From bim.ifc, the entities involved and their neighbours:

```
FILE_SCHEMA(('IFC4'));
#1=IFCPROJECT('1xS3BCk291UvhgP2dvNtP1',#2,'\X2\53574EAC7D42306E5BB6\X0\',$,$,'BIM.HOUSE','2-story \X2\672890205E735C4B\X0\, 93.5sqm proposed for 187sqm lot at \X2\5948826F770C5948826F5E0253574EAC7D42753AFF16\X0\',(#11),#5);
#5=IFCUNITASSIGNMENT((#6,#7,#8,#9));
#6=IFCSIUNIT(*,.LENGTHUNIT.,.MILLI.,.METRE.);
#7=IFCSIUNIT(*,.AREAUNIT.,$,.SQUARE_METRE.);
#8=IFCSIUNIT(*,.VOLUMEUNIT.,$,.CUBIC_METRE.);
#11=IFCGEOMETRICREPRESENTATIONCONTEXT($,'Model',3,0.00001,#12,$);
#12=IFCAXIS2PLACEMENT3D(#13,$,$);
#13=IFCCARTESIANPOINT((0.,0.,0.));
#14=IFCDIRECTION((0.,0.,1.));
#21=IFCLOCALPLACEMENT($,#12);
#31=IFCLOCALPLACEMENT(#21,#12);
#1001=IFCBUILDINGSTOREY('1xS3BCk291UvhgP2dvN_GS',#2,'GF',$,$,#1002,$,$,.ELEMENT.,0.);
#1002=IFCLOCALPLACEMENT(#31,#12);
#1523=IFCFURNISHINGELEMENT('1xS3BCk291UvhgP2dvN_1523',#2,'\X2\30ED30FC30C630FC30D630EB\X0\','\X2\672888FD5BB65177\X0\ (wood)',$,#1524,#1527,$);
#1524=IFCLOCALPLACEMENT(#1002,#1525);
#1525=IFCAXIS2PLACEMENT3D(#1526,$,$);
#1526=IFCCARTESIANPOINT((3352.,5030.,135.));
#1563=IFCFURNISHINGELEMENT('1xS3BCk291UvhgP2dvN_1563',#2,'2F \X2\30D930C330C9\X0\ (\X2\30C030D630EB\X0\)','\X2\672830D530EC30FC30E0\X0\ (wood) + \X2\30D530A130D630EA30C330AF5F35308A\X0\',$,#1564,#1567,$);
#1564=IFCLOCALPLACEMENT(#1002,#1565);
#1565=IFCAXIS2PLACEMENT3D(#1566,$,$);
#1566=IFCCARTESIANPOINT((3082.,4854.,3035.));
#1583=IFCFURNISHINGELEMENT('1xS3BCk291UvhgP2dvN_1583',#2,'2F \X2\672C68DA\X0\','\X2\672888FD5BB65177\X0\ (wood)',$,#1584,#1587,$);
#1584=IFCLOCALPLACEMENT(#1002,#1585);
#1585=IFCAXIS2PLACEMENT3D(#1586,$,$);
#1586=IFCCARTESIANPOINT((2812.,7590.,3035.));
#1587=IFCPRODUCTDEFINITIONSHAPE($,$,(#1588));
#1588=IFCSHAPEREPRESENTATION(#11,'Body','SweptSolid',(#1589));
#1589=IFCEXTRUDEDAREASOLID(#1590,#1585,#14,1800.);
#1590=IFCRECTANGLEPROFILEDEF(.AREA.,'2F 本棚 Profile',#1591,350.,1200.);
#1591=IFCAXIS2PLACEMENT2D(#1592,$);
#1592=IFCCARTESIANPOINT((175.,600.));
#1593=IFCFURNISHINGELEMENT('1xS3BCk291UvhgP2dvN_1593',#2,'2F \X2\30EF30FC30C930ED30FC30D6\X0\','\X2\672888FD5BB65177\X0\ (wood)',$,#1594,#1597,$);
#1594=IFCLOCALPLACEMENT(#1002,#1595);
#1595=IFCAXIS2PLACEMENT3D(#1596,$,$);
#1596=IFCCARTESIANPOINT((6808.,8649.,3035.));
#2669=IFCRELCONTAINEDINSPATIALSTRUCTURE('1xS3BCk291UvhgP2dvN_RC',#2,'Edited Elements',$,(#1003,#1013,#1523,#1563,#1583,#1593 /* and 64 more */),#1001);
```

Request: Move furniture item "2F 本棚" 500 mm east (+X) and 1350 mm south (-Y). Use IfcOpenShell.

```python
import ifcopenshell
import ifcopenshell.api.geometry
import ifcopenshell.util.placement

model = ifcopenshell.open("bim.ifc")

item = model.by_guid("1xS3BCk291UvhgP2dvN_1583")
matrix = ifcopenshell.util.placement.get_local_placement(item.ObjectPlacement)
matrix[0, 3] += 500.0
matrix[1, 3] -= 1350.0
ifcopenshell.api.geometry.edit_object_placement(model, product=item, matrix=matrix, is_si=False)

print(ifcopenshell.util.placement.get_local_placement(item.ObjectPlacement).round(3) + 0.0)

model.write("bim_updated.ifc")
```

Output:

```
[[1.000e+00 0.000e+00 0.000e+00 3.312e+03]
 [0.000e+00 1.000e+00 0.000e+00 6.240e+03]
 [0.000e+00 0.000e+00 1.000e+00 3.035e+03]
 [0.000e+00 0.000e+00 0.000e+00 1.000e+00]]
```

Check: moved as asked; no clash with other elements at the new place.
